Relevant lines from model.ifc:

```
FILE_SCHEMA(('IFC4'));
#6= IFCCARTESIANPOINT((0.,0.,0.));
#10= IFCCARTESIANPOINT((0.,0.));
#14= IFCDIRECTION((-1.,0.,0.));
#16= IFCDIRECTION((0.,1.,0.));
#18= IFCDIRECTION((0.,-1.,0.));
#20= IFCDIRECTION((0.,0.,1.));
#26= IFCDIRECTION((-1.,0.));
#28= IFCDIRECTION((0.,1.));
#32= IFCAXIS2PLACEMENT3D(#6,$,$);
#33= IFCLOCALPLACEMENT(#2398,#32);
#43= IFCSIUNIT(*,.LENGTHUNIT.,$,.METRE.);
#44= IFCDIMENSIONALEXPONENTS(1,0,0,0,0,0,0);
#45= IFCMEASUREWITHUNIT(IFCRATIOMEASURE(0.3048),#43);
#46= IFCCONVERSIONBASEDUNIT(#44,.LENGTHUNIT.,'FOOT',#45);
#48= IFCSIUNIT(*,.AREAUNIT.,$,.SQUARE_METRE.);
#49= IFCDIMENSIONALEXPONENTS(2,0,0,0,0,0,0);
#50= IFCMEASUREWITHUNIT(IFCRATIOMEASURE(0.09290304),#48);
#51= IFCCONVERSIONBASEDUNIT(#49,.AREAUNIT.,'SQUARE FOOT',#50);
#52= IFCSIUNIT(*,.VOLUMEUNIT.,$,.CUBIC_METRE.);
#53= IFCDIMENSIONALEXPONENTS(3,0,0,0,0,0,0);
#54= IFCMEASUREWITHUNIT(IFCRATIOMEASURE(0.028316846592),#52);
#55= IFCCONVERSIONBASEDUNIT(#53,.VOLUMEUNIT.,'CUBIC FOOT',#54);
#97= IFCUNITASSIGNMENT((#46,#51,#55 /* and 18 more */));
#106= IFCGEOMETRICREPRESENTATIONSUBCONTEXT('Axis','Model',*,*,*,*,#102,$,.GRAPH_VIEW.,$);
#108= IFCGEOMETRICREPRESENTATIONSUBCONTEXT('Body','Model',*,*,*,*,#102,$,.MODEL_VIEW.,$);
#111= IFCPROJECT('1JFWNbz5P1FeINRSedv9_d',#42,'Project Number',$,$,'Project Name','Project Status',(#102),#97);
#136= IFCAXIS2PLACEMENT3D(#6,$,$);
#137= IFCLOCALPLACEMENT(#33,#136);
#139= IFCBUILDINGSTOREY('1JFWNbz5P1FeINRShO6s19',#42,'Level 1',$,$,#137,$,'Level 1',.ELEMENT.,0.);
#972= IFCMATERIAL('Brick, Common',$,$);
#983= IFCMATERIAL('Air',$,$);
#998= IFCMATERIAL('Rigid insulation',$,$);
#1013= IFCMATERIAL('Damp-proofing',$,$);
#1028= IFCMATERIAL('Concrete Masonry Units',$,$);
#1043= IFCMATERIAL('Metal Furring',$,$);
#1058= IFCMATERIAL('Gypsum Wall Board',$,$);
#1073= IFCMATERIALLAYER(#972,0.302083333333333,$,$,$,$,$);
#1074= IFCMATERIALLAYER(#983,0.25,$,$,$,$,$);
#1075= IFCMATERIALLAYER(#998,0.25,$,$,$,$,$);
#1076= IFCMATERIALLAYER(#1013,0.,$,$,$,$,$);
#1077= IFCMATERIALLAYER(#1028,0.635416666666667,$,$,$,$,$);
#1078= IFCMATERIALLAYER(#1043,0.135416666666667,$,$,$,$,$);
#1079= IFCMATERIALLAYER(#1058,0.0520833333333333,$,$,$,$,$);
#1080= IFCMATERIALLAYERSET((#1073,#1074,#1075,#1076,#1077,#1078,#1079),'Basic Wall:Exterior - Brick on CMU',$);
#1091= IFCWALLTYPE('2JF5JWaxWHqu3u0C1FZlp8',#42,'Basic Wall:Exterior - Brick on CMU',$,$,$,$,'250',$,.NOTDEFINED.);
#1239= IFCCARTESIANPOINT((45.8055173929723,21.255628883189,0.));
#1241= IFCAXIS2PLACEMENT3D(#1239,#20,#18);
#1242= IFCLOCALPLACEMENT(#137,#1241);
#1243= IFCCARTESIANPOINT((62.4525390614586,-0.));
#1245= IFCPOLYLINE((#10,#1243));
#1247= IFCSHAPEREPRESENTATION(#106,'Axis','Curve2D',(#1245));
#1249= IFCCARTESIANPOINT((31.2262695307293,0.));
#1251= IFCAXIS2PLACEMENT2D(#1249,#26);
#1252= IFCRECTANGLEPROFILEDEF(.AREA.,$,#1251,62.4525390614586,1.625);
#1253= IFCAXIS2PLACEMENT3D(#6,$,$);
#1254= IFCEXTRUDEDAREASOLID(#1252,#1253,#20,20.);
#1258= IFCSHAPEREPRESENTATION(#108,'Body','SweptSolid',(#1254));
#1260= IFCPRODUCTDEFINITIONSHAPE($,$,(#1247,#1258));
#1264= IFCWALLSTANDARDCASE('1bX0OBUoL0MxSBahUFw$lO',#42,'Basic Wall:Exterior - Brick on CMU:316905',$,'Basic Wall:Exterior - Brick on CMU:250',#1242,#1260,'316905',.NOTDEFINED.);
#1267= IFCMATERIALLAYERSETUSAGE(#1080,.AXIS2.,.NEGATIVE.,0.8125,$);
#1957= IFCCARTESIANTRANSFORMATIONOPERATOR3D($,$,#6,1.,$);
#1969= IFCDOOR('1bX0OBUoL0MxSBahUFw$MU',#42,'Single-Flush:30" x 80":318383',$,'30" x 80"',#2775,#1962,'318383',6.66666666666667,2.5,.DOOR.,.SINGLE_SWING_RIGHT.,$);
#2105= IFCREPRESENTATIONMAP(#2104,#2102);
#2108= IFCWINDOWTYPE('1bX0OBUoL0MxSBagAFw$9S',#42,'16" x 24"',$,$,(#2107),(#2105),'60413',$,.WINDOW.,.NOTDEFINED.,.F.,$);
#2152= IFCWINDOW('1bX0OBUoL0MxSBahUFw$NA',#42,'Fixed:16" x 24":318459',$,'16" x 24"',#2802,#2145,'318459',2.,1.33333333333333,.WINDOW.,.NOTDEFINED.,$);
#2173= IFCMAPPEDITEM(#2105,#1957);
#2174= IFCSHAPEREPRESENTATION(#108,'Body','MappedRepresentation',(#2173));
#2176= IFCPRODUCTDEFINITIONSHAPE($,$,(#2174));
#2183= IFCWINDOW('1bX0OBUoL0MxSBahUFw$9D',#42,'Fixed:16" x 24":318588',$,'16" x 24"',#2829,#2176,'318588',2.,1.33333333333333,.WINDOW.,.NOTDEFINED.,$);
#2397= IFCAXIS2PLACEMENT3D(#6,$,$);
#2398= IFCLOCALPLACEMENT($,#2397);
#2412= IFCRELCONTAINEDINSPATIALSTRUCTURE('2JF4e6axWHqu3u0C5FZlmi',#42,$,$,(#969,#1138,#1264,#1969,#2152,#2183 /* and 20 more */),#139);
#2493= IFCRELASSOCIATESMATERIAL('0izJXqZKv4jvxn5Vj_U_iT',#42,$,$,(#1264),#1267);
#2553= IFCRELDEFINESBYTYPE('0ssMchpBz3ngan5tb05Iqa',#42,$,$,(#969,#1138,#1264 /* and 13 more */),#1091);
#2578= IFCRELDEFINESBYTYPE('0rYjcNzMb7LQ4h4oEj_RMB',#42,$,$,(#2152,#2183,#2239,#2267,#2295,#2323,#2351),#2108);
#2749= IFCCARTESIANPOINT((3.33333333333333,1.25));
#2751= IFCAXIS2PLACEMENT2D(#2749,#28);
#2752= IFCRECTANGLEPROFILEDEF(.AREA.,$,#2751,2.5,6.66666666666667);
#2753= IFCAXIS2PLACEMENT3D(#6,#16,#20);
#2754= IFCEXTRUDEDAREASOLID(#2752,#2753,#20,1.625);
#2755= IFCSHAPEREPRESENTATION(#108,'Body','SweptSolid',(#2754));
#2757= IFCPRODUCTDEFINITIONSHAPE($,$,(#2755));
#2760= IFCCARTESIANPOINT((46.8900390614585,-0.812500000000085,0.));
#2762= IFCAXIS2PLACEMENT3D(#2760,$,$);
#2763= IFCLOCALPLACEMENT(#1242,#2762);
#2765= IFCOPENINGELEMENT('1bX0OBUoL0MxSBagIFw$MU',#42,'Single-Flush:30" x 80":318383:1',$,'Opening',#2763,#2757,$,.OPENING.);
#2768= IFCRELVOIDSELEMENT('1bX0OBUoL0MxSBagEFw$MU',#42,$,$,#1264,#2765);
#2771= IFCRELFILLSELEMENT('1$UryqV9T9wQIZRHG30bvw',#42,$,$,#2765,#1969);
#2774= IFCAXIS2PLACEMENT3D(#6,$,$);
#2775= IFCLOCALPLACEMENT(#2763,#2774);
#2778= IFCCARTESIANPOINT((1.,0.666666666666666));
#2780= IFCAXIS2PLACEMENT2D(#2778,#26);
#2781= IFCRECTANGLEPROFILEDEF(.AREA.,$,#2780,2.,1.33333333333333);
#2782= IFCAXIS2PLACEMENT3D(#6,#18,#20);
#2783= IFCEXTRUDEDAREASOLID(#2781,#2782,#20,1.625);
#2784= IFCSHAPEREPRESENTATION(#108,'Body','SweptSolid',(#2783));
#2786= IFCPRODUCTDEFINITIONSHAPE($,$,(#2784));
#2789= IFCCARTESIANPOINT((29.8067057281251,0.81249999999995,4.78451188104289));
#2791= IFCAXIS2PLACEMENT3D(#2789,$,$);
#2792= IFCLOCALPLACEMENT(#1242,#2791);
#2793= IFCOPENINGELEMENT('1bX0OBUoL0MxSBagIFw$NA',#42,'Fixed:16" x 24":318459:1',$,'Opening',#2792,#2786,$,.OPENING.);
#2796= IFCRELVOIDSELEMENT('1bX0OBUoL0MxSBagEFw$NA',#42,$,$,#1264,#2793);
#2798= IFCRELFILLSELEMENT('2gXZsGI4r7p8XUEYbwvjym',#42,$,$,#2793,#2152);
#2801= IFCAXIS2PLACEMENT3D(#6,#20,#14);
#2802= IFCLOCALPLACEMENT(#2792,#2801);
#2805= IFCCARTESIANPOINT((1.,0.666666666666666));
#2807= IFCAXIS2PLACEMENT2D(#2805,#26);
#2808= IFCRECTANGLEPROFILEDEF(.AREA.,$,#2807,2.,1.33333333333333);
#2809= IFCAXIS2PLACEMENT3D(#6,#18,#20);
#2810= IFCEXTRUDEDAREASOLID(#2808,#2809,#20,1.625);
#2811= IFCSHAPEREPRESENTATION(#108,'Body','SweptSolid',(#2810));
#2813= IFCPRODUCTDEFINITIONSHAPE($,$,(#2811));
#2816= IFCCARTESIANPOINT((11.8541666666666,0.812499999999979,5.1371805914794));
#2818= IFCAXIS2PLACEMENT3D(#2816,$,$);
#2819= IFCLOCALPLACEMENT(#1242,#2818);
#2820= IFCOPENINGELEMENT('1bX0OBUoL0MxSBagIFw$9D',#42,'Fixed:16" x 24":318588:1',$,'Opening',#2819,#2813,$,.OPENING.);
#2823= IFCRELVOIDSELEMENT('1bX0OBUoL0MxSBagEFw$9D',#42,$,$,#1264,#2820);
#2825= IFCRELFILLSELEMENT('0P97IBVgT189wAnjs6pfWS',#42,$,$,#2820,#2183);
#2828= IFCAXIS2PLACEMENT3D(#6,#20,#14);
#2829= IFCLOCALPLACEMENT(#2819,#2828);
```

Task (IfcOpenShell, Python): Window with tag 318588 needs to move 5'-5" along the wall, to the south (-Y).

```python
import ifcopenshell
import ifcopenshell.api.geometry
import ifcopenshell.util.placement
import ifcopenshell.util.unit

model = ifcopenshell.open("model.ifc")
unit_scale = ifcopenshell.util.unit.calculate_unit_scale(model)

window = model.by_guid("1bX0OBUoL0MxSBahUFw$9D")
opening = window.FillsVoids[0].RelatingOpeningElement
wall = opening.VoidsElements[0].RelatingBuildingElement

wall_matrix = ifcopenshell.util.placement.get_local_placement(wall.ObjectPlacement)
shift = wall_matrix[:3, 0] * 65 * 0.0254 / unit_scale
before = ifcopenshell.util.placement.get_local_placement(window.ObjectPlacement)[:3, 3].copy()

# The window is placed relative to its opening, so it follows when the opening moves.
matrix = ifcopenshell.util.placement.get_local_placement(opening.ObjectPlacement)
matrix[:3, 3] += shift
ifcopenshell.api.geometry.edit_object_placement(
    model, product=opening, matrix=matrix, is_si=False, should_transform_children=True
)

after = ifcopenshell.util.placement.get_local_placement(window.ObjectPlacement)[:3, 3]
print("window moved by", (after - before).round(3) + 0.0)

model.write("model_rev.ifc")
```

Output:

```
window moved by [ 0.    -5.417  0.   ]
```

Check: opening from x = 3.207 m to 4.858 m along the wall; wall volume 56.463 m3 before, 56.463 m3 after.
